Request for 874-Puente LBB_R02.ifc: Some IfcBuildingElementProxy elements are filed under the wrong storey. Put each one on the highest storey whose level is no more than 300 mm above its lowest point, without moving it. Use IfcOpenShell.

First a look at what the model holds.

```python
import ifcopenshell
import ifcopenshell.util.element
import ifcopenshell.util.placement

model = ifcopenshell.open("874-Puente LBB_R02.ifc")
print(model.schema)
for storey in model.by_type("IfcBuildingStorey"):
    level = ifcopenshell.util.placement.get_storey_elevation(storey)
    count = sum(e.is_a("IfcBuildingElementProxy") for e in ifcopenshell.util.element.get_contained(storey))
    print(storey.id(), storey.Name, round(level, 3), count, sep=" | ")
```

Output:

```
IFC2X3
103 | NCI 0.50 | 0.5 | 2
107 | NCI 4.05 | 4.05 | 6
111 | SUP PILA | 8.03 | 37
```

```python
import ifcopenshell
import ifcopenshell.api.spatial
import ifcopenshell.geom
import ifcopenshell.util.element
import ifcopenshell.util.placement
import ifcopenshell.util.shape
import ifcopenshell.util.unit

model = ifcopenshell.open("874-Puente LBB_R02.ifc")
unit_scale = ifcopenshell.util.unit.calculate_unit_scale(model)
settings = ifcopenshell.geom.settings()

levels = sorted(
    ((ifcopenshell.util.placement.get_storey_elevation(s) * unit_scale, s) for s in model.by_type("IfcBuildingStorey")),
    key=lambda pair: pair[0],
)

for e in model.by_type("IfcBuildingElementProxy"):
    current = e.ContainedInStructure[0].RelatingStructure if e.ContainedInStructure else None
    if current is None or not current.is_a("IfcBuildingStorey"):
        continue
    shape = ifcopenshell.geom.create_shape(settings, e)
    bottom = ifcopenshell.util.shape.get_shape_bottom_elevation(shape, shape.geometry)
    below = [s for level, s in levels if level <= bottom + 0.3]
    storey = below[-1] if below else levels[0][1]
    if storey != current:
        # assign_container keeps the world position.
        ifcopenshell.api.spatial.assign_container(model, products=[e], relating_structure=storey)
        print(e.id(), current.Name, "->", storey.Name)

model.write("874-Puente LBB_R02-out.ifc")
```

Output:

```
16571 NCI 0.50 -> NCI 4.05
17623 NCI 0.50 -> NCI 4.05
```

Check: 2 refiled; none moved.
